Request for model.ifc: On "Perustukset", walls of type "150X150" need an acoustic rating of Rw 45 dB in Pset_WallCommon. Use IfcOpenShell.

First a look at what the model holds.

```python
import ifcopenshell
import ifcopenshell.util.element

model = ifcopenshell.open("model.ifc")
print(model.schema)
storey = next(s for s in model.by_type("IfcBuildingStorey") if s.Name == "Perustukset")
walls = [e for e in ifcopenshell.util.element.get_decomposition(storey) if e.is_a("IfcWall")]
seen = {}
for e in walls:
    element_type = ifcopenshell.util.element.get_type(e)
    key = (element_type.Name if element_type != e and element_type else None, ifcopenshell.util.element.get_pset(e, "Pset_WallCommon", "AcousticRating"))
    seen[key] = seen.get(key, 0) + 1
for (name, value), count in sorted(seen.items(), key=str):
    print(count, "x", name, "|", value)
```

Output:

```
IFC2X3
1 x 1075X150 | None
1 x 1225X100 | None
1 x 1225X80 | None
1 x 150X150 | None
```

```python
import ifcopenshell
import ifcopenshell.api.pset
import ifcopenshell.util.element

model = ifcopenshell.open("model.ifc")

storey = next(s for s in model.by_type("IfcBuildingStorey") if s.Name == "Perustukset")
walls = [e for e in ifcopenshell.util.element.get_decomposition(storey) if e.is_a("IfcWall")]

count = 0
for e in walls:
    element_type = ifcopenshell.util.element.get_type(e)
    if element_type in (None, e) or element_type.Name != "150X150":
        continue
    # add_pset returns the element's existing set when there is one.
    pset = ifcopenshell.api.pset.add_pset(model, product=e, name="Pset_WallCommon")
    ifcopenshell.api.pset.edit_pset(model, pset=pset, properties={"AcousticRating": "Rw 45 dB"})
    count += 1

print(count, "walls updated")

model.write("model-out.ifc")
```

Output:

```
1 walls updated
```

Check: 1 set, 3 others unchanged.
